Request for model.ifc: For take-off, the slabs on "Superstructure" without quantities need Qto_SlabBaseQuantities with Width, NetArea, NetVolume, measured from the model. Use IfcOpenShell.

First a look at what the model holds.

```python
import ifcopenshell
import ifcopenshell.util.element
import ifcopenshell.util.unit

model = ifcopenshell.open("model.ifc")
print(model.schema)
for unit_type in ("LENGTHUNIT", "AREAUNIT", "VOLUMEUNIT"):
    print(unit_type, ifcopenshell.util.unit.calculate_unit_scale(model, unit_type))
storey = next(s for s in model.by_type("IfcBuildingStorey") if s.Name == "Superstructure")
slabs = [e for e in ifcopenshell.util.element.get_decomposition(storey) if e.is_a("IfcSlab")]
for e in sorted(slabs, key=lambda e: e.id()):
    print(e.id(), e.is_a(), e.Name, list(ifcopenshell.util.element.get_psets(e, qtos_only=True)), sep=" | ")
```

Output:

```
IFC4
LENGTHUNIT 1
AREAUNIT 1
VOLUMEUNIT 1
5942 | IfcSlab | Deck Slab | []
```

```python
import ifcopenshell
import ifcopenshell.api.pset
import ifcopenshell.geom
import ifcopenshell.util.element
import ifcopenshell.util.shape
import ifcopenshell.util.unit

model = ifcopenshell.open("model.ifc")
unit_scale = ifcopenshell.util.unit.calculate_unit_scale(model)
area_scale = ifcopenshell.util.unit.calculate_unit_scale(model, "AREAUNIT")
volume_scale = ifcopenshell.util.unit.calculate_unit_scale(model, "VOLUMEUNIT")
settings = ifcopenshell.geom.settings()

storey = next(s for s in model.by_type("IfcBuildingStorey") if s.Name == "Superstructure")
slabs = [e for e in ifcopenshell.util.element.get_decomposition(storey) if e.is_a("IfcSlab")]

for e in sorted(slabs, key=lambda e: e.id()):
    if ifcopenshell.util.element.get_psets(e, qtos_only=True, should_inherit=False):
        continue
    # Geometry comes back in metres, in the element's own axes.
    shape = ifcopenshell.geom.create_shape(settings, e)
    values = {
        "Width": ifcopenshell.util.shape.get_z(shape.geometry) / unit_scale,
        "NetArea": ifcopenshell.util.shape.get_footprint_area(shape.geometry) / area_scale,
        "NetVolume": ifcopenshell.util.shape.get_volume(shape.geometry) / volume_scale,
    }
    qto = ifcopenshell.api.pset.add_qto(model, product=e, name="Qto_SlabBaseQuantities")
    ifcopenshell.api.pset.edit_qto(model, qto=qto, properties=values)
    print(e.id(), {k: round(v, 3) for k, v in values.items()})

model.write("model_edited.ifc")
```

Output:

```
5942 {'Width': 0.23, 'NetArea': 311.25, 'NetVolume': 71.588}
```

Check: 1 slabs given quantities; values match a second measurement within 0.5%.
